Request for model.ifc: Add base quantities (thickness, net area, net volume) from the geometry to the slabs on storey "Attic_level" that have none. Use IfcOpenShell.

First a look at what the model holds.

```python
import ifcopenshell
import ifcopenshell.util.element
import ifcopenshell.util.unit

model = ifcopenshell.open("model.ifc")
print(model.schema)
for unit_type in ("LENGTHUNIT", "AREAUNIT", "VOLUMEUNIT"):
    print(unit_type, ifcopenshell.util.unit.calculate_unit_scale(model, unit_type))
storey = next(s for s in model.by_type("IfcBuildingStorey") if s.Name == "Attic_level")
slabs = [e for e in ifcopenshell.util.element.get_decomposition(storey) if e.is_a("IfcSlab")]
for e in sorted(slabs, key=lambda e: e.id()):
    print(e.id(), e.is_a(), e.Name, list(ifcopenshell.util.element.get_psets(e, qtos_only=True)), sep=" | ")
```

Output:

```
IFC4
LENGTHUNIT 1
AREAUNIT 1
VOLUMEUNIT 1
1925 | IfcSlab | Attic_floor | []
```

```python
import ifcopenshell
import ifcopenshell.api.pset
import ifcopenshell.geom
import ifcopenshell.util.element
import ifcopenshell.util.shape
import ifcopenshell.util.unit

model = ifcopenshell.open("model.ifc")
unit_scale = ifcopenshell.util.unit.calculate_unit_scale(model)
area_scale = ifcopenshell.util.unit.calculate_unit_scale(model, "AREAUNIT")
volume_scale = ifcopenshell.util.unit.calculate_unit_scale(model, "VOLUMEUNIT")
settings = ifcopenshell.geom.settings()

storey = next(s for s in model.by_type("IfcBuildingStorey") if s.Name == "Attic_level")
slabs = [e for e in ifcopenshell.util.element.get_decomposition(storey) if e.is_a("IfcSlab")]

for e in sorted(slabs, key=lambda e: e.id()):
    if ifcopenshell.util.element.get_psets(e, qtos_only=True, should_inherit=False):
        continue
    # Geometry comes back in metres, in the element's own axes.
    shape = ifcopenshell.geom.create_shape(settings, e)
    values = {
        "Width": ifcopenshell.util.shape.get_z(shape.geometry) / unit_scale,
        "NetArea": ifcopenshell.util.shape.get_footprint_area(shape.geometry) / area_scale,
        "NetVolume": ifcopenshell.util.shape.get_volume(shape.geometry) / volume_scale,
    }
    qto = ifcopenshell.api.pset.add_qto(model, product=e, name="Qto_SlabBaseQuantities")
    ifcopenshell.api.pset.edit_qto(model, qto=qto, properties=values)
    print(e.id(), {k: round(v, 3) for k, v in values.items()})

model.write("model-out.ifc")
```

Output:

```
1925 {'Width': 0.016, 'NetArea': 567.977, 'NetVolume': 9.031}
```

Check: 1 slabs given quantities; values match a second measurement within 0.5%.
